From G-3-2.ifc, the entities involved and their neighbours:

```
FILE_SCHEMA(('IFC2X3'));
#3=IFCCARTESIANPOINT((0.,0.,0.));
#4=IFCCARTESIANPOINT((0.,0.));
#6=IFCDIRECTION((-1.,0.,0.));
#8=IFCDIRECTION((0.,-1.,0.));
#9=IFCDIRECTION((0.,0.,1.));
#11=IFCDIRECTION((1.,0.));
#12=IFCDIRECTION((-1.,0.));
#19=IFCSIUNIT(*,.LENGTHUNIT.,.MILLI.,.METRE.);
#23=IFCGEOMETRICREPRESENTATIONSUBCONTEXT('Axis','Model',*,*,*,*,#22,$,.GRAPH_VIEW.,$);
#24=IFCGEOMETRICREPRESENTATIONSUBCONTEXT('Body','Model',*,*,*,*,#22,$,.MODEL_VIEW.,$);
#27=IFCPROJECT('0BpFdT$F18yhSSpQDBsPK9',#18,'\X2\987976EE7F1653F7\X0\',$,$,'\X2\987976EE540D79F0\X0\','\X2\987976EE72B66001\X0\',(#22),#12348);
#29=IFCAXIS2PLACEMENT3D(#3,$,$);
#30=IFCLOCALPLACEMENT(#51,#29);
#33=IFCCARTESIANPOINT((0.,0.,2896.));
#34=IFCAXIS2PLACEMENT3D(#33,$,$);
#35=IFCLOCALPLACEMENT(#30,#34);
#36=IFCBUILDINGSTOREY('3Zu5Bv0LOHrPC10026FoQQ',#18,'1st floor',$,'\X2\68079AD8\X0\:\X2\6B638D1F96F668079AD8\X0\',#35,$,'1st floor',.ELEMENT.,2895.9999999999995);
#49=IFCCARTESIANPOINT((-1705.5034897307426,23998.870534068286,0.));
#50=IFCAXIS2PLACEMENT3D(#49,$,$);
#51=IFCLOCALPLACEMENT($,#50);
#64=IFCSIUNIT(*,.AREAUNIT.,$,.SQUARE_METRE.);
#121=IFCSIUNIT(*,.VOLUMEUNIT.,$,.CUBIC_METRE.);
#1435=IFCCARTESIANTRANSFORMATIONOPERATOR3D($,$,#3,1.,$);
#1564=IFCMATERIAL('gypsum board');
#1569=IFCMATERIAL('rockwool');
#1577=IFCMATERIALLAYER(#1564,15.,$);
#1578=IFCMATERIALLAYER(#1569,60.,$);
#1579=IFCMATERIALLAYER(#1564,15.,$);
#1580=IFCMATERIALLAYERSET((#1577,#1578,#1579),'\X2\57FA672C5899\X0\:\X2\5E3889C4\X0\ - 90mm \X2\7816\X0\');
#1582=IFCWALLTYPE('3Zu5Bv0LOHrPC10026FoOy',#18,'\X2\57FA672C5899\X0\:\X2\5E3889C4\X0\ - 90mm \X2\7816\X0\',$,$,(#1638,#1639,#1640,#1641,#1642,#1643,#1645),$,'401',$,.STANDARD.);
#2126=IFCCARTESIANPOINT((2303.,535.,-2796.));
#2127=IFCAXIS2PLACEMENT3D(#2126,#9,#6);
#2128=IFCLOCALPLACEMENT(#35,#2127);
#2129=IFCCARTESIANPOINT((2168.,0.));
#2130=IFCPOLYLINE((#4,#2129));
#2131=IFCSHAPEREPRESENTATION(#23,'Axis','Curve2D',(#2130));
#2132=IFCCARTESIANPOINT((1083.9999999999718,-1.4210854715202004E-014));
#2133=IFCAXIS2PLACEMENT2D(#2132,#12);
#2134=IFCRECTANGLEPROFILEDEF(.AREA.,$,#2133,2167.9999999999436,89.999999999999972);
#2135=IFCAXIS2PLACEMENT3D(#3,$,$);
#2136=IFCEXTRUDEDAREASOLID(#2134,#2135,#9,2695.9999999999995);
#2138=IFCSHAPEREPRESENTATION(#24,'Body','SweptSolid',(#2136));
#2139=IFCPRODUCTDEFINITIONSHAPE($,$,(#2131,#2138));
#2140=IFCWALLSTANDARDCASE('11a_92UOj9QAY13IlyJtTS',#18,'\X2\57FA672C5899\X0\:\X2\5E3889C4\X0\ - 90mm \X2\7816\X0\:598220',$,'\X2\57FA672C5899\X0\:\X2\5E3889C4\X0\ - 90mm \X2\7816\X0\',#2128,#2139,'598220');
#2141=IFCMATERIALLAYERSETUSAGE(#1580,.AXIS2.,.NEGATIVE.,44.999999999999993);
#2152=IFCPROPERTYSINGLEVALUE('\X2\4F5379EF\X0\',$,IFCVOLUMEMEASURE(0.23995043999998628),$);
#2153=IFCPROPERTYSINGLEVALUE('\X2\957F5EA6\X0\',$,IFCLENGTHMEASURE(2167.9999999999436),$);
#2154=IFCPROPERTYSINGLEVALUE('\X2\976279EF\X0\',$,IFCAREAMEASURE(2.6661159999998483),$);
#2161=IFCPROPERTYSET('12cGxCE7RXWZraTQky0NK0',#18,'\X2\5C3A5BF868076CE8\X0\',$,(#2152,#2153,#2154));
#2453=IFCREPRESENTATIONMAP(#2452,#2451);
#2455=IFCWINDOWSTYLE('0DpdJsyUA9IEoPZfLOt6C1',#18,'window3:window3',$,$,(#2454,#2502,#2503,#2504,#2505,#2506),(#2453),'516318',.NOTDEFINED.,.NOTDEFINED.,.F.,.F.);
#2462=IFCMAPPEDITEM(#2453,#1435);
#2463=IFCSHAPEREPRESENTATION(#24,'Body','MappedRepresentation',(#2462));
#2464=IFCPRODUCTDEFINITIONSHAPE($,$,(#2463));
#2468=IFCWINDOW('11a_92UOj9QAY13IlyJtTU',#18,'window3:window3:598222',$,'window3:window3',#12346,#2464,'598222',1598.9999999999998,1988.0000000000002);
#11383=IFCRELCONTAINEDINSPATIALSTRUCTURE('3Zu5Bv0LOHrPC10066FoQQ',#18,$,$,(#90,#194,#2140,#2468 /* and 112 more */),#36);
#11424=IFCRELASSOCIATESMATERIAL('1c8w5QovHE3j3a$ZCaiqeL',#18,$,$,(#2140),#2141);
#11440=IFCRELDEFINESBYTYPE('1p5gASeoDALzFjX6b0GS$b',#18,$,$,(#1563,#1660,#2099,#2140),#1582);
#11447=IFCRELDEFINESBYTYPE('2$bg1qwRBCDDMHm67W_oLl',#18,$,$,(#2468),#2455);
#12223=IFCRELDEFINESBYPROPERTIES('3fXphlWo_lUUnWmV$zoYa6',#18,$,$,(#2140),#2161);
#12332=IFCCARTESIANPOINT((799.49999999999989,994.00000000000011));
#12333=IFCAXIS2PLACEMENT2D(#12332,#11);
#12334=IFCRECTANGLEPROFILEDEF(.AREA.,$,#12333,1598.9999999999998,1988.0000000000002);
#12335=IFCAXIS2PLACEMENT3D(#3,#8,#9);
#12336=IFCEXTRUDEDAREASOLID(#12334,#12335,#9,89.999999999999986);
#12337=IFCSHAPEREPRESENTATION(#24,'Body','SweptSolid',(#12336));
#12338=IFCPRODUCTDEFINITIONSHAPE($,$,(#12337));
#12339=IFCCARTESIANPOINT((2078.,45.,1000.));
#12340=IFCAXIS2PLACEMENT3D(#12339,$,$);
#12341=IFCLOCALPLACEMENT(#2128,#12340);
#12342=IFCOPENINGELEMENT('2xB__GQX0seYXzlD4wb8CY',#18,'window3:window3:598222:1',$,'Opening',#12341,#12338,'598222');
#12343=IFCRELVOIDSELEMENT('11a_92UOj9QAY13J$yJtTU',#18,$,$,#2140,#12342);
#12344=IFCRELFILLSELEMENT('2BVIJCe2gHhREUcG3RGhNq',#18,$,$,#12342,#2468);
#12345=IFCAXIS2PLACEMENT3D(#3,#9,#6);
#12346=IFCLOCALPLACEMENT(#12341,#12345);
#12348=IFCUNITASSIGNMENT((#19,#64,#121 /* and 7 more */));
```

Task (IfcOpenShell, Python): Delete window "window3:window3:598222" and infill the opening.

```python
import ifcopenshell
import ifcopenshell.api.feature
import ifcopenshell.api.pset
import ifcopenshell.api.root
import ifcopenshell.geom
import ifcopenshell.util.element
import ifcopenshell.util.shape
import ifcopenshell.util.unit

model = ifcopenshell.open("G-3-2.ifc")
area_scale = ifcopenshell.util.unit.calculate_unit_scale(model, "AREAUNIT")
volume_scale = ifcopenshell.util.unit.calculate_unit_scale(model, "VOLUMEUNIT")
settings = ifcopenshell.geom.settings()


def volume(element):
    """Net volume in cubic metres, openings subtracted."""
    shape = ifcopenshell.geom.create_shape(settings, element)
    return ifcopenshell.util.shape.get_volume(shape.geometry)


window = model.by_guid("11a_92UOj9QAY13IlyJtTU")
opening = window.FillsVoids[0].RelatingOpeningElement
wall = opening.VoidsElements[0].RelatingBuildingElement
before = volume(wall)

ifcopenshell.api.root.remove_product(model, product=window)
ifcopenshell.api.feature.remove_feature(model, feature=opening)

after = volume(wall)
thickness = 0.09  # wall thickness in metres

# Update the wall's stored quantities.
pset = model.by_id(ifcopenshell.util.element.get_pset(wall, "尺寸标注", should_inherit=False)["id"])
ifcopenshell.api.pset.edit_pset(model, pset=pset, properties={
    "体积": model.create_entity("IfcVolumeMeasure", after / volume_scale),
    "面积": model.create_entity("IfcAreaMeasure", after / thickness / area_scale),
})

print(f"wall volume {before:.3f} -> {after:.3f} m3")

model.write("G-3-2_rev.ifc")
```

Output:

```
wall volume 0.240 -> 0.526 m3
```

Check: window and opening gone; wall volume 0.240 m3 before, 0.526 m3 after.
